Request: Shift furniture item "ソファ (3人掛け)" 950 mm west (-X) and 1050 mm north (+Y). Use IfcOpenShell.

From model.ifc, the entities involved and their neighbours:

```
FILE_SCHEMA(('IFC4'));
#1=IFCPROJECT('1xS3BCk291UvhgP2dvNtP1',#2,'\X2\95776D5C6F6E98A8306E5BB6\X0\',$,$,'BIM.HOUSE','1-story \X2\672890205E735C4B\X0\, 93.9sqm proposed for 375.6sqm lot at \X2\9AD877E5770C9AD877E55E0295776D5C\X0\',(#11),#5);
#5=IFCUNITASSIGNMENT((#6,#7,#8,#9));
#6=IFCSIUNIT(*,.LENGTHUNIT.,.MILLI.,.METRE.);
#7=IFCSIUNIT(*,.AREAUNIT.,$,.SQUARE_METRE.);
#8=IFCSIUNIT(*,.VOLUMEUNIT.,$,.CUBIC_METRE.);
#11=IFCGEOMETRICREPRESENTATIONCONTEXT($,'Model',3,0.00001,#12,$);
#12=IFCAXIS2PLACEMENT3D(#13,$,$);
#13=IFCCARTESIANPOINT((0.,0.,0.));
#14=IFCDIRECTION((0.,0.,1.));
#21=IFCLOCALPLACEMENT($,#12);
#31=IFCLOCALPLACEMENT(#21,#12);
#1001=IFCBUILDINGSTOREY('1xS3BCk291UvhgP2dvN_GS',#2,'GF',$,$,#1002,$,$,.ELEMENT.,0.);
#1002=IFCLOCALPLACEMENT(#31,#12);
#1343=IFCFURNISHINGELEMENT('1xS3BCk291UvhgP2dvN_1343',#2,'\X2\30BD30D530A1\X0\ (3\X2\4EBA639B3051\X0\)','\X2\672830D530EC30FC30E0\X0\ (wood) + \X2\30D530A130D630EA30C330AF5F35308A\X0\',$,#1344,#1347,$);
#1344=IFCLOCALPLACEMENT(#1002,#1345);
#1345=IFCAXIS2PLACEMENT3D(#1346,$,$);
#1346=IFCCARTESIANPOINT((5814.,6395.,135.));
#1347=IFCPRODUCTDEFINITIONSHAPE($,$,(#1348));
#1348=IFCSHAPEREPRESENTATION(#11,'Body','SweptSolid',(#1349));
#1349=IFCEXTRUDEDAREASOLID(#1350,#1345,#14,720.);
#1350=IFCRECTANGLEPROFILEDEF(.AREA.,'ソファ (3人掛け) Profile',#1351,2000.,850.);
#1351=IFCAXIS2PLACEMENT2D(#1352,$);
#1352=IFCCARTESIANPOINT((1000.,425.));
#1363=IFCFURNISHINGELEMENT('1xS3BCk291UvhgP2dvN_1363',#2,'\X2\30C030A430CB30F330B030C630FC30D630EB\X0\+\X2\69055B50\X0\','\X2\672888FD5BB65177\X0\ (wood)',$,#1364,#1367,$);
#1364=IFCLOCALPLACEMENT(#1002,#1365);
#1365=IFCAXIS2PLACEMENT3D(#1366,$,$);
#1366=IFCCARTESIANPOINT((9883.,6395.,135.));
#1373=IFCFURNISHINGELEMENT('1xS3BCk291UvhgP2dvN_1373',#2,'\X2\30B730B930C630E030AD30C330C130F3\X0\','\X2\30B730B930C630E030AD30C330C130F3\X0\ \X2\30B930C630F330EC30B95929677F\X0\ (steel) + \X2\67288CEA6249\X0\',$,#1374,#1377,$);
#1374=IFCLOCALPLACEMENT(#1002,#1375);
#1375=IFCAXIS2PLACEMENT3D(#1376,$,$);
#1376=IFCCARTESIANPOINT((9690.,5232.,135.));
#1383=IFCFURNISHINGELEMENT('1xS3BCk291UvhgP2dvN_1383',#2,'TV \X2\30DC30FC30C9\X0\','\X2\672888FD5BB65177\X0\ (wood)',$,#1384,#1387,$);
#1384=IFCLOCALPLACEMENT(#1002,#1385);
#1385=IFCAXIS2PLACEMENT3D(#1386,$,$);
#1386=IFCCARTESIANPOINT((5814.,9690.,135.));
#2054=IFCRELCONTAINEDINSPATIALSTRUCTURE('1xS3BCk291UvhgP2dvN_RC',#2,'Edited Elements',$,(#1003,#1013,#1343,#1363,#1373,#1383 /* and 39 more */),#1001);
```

```python
import ifcopenshell
import ifcopenshell.api.geometry
import ifcopenshell.util.placement
import ifcopenshell.util.unit

model = ifcopenshell.open("model.ifc")
unit_scale = ifcopenshell.util.unit.calculate_unit_scale(model)

item = model.by_guid("1xS3BCk291UvhgP2dvN_1343")
matrix = ifcopenshell.util.placement.get_local_placement(item.ObjectPlacement)
matrix[0, 3] -= 0.95 / unit_scale
matrix[1, 3] += 1.05 / unit_scale
ifcopenshell.api.geometry.edit_object_placement(model, product=item, matrix=matrix, is_si=False)

print(ifcopenshell.util.placement.get_local_placement(item.ObjectPlacement).round(3) + 0.0)

model.write("model_updated.ifc")
```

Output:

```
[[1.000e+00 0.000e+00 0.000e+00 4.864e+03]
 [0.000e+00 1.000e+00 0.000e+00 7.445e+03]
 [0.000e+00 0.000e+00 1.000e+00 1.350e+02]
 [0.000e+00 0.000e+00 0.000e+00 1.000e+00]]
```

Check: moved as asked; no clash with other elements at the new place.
